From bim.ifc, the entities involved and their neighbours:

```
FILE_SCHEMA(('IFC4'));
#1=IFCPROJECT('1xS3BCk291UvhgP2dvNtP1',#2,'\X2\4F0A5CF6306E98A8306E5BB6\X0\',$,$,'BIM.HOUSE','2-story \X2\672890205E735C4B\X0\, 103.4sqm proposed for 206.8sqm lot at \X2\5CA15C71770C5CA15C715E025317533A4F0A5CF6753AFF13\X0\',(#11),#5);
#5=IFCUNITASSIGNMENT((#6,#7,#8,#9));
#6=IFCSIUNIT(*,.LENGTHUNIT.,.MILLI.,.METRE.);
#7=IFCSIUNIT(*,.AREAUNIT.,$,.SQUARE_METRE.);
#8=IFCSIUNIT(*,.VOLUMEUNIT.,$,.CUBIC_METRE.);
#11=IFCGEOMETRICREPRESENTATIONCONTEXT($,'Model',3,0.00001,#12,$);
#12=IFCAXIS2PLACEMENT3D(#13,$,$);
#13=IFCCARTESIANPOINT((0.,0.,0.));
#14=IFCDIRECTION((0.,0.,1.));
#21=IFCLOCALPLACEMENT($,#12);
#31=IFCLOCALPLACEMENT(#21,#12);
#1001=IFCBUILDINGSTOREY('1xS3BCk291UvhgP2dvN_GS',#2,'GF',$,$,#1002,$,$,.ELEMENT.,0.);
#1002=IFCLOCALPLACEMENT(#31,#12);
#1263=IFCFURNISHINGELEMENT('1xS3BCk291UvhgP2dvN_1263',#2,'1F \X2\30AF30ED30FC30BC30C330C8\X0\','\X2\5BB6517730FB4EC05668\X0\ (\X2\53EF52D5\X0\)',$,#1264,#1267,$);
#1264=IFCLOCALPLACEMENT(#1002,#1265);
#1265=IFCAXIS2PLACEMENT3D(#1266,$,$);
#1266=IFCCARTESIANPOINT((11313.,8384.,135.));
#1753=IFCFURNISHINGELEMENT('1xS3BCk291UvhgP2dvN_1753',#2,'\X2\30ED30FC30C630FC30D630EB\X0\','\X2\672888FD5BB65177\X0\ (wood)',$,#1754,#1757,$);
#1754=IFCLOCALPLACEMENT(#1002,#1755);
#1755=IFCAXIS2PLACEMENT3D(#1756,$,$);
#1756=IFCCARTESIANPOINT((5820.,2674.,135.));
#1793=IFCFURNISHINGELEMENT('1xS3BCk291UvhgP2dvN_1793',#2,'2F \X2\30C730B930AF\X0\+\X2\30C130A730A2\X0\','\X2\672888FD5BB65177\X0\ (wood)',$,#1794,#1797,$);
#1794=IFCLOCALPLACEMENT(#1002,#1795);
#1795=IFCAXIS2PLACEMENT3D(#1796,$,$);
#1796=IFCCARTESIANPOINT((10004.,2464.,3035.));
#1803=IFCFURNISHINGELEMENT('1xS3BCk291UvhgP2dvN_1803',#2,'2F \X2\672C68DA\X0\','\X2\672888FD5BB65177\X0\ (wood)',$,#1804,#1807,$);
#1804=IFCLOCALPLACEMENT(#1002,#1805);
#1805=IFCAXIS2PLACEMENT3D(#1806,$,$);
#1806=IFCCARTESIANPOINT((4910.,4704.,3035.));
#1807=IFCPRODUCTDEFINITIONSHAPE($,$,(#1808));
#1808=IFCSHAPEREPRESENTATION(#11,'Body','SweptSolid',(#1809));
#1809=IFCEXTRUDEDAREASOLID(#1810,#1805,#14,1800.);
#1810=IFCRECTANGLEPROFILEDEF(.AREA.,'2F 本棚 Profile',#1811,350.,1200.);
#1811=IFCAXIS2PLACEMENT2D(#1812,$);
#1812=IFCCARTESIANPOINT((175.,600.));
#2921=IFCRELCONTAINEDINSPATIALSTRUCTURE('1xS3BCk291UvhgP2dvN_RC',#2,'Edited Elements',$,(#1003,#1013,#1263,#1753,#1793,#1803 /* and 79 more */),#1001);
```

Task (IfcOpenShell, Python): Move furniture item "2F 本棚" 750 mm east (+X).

```python
import ifcopenshell
import ifcopenshell.api.geometry
import ifcopenshell.util.placement

model = ifcopenshell.open("bim.ifc")

item = model.by_guid("1xS3BCk291UvhgP2dvN_1803")
matrix = ifcopenshell.util.placement.get_local_placement(item.ObjectPlacement)
matrix[0, 3] += 750.0
ifcopenshell.api.geometry.edit_object_placement(model, product=item, matrix=matrix, is_si=False)

print(ifcopenshell.util.placement.get_local_placement(item.ObjectPlacement).round(3) + 0.0)

model.write("bim_edited.ifc")
```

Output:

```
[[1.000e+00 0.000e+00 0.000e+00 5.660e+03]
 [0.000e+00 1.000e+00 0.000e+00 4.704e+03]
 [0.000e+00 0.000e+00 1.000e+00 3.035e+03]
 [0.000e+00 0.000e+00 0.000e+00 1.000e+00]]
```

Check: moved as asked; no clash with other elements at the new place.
